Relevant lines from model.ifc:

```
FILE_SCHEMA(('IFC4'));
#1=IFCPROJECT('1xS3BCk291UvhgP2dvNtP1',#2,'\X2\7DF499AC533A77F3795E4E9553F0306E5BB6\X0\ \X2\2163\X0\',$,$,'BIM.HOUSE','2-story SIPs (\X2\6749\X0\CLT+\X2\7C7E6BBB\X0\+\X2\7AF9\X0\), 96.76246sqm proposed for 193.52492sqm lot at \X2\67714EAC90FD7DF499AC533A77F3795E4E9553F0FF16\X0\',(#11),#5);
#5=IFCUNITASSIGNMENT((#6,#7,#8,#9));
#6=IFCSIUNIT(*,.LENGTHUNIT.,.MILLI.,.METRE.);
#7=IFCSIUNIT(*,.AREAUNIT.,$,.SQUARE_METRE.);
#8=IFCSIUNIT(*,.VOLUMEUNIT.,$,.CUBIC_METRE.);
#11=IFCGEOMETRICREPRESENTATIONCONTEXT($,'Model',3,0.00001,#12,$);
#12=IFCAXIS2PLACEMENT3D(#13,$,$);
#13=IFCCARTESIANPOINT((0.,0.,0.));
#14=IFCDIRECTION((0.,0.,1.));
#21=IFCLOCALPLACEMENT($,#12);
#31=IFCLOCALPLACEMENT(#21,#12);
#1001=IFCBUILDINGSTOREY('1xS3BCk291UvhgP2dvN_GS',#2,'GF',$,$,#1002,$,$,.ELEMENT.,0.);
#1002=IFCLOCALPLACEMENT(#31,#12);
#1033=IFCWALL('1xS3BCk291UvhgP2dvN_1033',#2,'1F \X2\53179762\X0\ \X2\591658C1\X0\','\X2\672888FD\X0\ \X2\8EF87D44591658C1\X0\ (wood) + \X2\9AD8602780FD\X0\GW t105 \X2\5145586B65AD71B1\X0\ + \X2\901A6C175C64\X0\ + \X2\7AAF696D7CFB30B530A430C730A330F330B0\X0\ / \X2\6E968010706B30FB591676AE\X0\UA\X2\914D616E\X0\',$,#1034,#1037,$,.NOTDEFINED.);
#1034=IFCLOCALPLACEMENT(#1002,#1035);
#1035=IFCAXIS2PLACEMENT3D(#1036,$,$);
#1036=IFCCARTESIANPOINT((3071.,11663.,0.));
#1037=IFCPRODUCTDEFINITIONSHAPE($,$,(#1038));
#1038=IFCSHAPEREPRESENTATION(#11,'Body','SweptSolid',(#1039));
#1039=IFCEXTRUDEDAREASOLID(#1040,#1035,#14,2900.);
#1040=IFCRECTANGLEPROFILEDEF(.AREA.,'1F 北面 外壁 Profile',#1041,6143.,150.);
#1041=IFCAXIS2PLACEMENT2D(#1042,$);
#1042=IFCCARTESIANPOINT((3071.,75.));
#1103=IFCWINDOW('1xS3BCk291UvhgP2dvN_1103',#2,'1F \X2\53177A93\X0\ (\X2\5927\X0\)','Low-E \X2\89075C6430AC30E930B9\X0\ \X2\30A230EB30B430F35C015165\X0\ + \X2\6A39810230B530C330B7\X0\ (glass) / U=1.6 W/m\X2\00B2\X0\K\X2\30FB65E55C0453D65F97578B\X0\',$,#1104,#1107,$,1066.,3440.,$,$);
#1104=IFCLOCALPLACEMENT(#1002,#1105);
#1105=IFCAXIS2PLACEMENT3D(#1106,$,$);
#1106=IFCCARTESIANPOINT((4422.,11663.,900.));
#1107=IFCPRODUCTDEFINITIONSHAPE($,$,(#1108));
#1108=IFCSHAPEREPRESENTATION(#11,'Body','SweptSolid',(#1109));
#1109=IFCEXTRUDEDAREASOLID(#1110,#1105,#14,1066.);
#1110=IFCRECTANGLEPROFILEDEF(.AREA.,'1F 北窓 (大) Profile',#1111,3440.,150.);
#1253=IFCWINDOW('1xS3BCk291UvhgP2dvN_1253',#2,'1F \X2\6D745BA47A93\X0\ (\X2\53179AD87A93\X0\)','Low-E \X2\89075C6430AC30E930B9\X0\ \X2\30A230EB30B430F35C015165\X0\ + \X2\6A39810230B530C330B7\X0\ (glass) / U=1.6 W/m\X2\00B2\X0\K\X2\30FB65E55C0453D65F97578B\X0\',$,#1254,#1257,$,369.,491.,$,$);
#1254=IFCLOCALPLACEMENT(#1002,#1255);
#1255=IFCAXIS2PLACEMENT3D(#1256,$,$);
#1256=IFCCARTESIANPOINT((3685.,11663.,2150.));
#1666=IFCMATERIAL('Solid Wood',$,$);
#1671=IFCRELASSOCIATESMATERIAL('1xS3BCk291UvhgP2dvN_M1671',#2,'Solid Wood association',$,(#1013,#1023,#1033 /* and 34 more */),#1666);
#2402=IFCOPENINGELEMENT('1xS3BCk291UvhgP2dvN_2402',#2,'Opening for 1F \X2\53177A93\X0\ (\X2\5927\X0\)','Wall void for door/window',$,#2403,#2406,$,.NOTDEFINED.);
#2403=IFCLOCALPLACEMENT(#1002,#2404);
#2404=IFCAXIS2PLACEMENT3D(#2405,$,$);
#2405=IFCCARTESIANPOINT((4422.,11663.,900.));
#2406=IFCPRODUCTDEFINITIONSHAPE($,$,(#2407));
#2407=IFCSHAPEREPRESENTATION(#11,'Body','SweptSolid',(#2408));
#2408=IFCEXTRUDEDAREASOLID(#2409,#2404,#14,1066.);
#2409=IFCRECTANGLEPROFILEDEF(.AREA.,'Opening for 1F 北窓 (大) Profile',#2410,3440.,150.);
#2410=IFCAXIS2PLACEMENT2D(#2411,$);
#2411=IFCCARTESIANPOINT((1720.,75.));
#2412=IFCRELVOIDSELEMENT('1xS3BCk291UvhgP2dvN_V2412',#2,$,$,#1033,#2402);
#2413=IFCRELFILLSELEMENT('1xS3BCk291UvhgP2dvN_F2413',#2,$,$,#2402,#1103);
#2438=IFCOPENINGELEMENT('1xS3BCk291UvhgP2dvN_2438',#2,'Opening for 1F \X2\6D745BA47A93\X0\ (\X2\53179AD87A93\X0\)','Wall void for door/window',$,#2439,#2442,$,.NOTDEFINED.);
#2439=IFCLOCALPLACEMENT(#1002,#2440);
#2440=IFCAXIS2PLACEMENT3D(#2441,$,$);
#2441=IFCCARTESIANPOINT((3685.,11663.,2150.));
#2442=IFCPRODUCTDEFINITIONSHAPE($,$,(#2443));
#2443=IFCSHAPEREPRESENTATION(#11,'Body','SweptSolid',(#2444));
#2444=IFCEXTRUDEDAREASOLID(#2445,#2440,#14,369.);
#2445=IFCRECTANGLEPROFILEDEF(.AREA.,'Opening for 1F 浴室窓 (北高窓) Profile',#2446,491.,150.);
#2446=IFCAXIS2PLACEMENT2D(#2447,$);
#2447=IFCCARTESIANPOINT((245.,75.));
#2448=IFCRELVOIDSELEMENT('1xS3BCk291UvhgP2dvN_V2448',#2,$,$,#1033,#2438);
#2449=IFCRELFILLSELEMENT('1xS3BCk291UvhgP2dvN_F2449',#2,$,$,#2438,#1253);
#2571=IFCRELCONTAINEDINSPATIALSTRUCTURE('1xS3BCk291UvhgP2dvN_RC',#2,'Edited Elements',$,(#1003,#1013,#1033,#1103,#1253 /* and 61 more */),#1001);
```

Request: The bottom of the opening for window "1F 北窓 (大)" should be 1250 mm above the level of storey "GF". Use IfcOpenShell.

```python
import numpy as np
import ifcopenshell
import ifcopenshell.api.geometry
import ifcopenshell.geom
import ifcopenshell.util.element
import ifcopenshell.util.placement
import ifcopenshell.util.shape
import ifcopenshell.util.unit

model = ifcopenshell.open("model.ifc")
unit_scale = ifcopenshell.util.unit.calculate_unit_scale(model)

window = model.by_id(1103)
opening = window.FillsVoids[0].RelatingOpeningElement
storey = ifcopenshell.util.element.get_container(window, ifc_class="IfcBuildingStorey")
level = ifcopenshell.util.placement.get_local_placement(storey.ObjectPlacement)[2, 3]

# The opening's origin need not be at the sill, so measure its lowest point.
shape = ifcopenshell.geom.create_shape(ifcopenshell.geom.settings(), opening)
bottom = ifcopenshell.util.shape.get_shape_bottom_elevation(shape, shape.geometry) / unit_scale
dz = level + 1.25 / unit_scale - bottom

shift = np.array([0.0, 0.0, dz])
# The window is not placed relative to its opening, so move both.
for product in (opening, window):
    matrix = ifcopenshell.util.placement.get_local_placement(product.ObjectPlacement)
    matrix[:3, 3] += shift
    ifcopenshell.api.geometry.edit_object_placement(model, product=product, matrix=matrix, is_si=False)

print(f"moved by {dz * unit_scale:+.3f} m")

model.write("model_rev.ifc")
```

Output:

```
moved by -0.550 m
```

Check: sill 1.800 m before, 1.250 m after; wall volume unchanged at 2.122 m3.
